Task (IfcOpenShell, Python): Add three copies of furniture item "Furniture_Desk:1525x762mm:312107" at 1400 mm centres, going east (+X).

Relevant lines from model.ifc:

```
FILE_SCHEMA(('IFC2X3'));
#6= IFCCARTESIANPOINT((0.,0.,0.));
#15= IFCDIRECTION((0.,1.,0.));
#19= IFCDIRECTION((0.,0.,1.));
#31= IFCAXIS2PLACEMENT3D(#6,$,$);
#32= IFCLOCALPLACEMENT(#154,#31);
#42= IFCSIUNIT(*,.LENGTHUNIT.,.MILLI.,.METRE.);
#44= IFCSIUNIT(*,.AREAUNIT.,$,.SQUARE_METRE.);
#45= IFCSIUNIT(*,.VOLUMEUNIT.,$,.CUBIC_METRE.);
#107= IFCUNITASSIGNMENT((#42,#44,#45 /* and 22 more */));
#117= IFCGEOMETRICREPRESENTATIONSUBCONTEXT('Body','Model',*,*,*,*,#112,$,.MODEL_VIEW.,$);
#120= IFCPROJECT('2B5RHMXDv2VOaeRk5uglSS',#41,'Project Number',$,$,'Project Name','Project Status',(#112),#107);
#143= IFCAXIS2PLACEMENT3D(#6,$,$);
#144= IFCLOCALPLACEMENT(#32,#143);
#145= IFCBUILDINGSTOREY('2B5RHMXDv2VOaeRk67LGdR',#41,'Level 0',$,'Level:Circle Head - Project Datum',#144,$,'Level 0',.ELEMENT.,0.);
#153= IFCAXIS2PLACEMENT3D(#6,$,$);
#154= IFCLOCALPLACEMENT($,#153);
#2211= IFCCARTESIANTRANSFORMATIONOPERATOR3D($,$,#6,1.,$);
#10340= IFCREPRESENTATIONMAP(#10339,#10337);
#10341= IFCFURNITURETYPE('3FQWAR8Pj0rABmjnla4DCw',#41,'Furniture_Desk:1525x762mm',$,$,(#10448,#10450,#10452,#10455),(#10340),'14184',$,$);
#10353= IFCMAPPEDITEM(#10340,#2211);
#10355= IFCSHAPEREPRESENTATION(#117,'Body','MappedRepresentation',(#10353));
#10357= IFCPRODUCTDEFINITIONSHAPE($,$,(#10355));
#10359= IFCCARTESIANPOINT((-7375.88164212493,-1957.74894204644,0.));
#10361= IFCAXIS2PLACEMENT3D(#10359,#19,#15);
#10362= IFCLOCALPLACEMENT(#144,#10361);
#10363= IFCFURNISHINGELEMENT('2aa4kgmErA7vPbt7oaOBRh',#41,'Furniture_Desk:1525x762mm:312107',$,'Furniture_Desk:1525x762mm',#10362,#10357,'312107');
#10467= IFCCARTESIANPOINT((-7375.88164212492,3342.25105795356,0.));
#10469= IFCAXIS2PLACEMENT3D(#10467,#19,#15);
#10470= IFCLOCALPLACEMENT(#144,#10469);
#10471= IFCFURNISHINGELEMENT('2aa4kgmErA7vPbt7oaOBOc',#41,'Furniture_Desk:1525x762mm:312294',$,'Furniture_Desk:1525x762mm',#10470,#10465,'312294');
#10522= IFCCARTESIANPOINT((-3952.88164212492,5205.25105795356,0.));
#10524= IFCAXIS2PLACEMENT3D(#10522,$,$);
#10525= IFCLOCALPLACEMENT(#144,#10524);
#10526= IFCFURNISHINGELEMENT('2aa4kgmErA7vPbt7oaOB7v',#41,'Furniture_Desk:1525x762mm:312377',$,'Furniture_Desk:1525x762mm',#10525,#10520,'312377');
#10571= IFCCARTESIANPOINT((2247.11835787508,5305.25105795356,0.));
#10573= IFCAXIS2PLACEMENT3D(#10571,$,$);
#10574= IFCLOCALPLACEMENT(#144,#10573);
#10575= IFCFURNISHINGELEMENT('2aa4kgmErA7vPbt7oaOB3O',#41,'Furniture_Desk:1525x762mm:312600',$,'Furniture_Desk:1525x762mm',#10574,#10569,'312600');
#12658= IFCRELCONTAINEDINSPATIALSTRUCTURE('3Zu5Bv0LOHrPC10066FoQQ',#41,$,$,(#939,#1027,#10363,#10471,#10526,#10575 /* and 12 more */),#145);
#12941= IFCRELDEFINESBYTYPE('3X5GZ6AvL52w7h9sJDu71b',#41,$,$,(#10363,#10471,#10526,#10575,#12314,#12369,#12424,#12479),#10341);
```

```python
import numpy as np
import ifcopenshell
import ifcopenshell.api.geometry
import ifcopenshell.api.root
import ifcopenshell.util.element
import ifcopenshell.util.placement
import ifcopenshell.util.unit

model = ifcopenshell.open("model.ifc")
unit_scale = ifcopenshell.util.unit.calculate_unit_scale(model)


def reuse_history(source, copy):
    """copy_class also copies each property set's owner history, people and application; keep the originals."""
    for rel in copy.IsDefinedBy:
        if rel.is_a("IfcRelDefinesByProperties") and (history := rel.RelatingPropertyDefinition.OwnerHistory):
            rel.RelatingPropertyDefinition.OwnerHistory = source.OwnerHistory
            ifcopenshell.util.element.remove_deep2(model, history)


source = model.by_guid("2aa4kgmErA7vPbt7oaOBRh")
base = ifcopenshell.util.placement.get_local_placement(source.ObjectPlacement)
step = np.array([1.0, 0.0, 0.0]) * 1.4 / unit_scale

for i in range(1, 4):
    copy = ifcopenshell.api.root.copy_class(model, product=source)
    copy.Representation = ifcopenshell.util.element.copy_deep(
        model, source.Representation, exclude=["IfcGeometricRepresentationContext", "IfcRepresentationMap"]
    )
    copy.Name = "Furniture_Desk:1525x762mm"
    copy.Tag = None
    reuse_history(source, copy)
    matrix = base.copy()
    matrix[:3, 3] += i * step
    print("added at", matrix[:3, 3].round(3) + 0.0)
    ifcopenshell.api.geometry.edit_object_placement(model, product=copy, matrix=matrix, is_si=False)

model.write("model_updated.ifc")
```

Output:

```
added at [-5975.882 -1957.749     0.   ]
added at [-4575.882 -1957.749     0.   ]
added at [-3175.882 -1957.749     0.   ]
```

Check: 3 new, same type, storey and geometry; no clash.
